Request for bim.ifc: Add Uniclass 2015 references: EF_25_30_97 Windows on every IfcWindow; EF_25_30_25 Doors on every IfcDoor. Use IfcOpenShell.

First a look at what the model holds.

```python
import ifcopenshell

model = ifcopenshell.open("bim.ifc")
print(model.schema)
print("classifications:", [c.Name for c in model.by_type("IfcClassification")])
for ifc_class in ("IfcDoor", "IfcRoof", "IfcStair", "IfcWall", "IfcWindow"):
    print(ifc_class, len(model.by_type(ifc_class)))
```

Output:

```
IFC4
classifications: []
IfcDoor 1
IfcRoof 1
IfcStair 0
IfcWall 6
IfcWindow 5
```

```python
import ifcopenshell
import ifcopenshell.api.classification

model = ifcopenshell.open("bim.ifc")

system = ifcopenshell.api.classification.add_classification(model, classification="Uniclass 2015")

codes = {
    "IfcWindow": ("EF_25_30_97", "Windows"),
    "IfcDoor": ("EF_25_30_25", "Doors"),
}
for ifc_class, (code, name) in codes.items():
    products = model.by_type(ifc_class)
    ifcopenshell.api.classification.add_reference(
        model, products=products, classification=system, identification=code, name=name
    )
    print(code, len(products))

model.write("bim_updated.ifc")
```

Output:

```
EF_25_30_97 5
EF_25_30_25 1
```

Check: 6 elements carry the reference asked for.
